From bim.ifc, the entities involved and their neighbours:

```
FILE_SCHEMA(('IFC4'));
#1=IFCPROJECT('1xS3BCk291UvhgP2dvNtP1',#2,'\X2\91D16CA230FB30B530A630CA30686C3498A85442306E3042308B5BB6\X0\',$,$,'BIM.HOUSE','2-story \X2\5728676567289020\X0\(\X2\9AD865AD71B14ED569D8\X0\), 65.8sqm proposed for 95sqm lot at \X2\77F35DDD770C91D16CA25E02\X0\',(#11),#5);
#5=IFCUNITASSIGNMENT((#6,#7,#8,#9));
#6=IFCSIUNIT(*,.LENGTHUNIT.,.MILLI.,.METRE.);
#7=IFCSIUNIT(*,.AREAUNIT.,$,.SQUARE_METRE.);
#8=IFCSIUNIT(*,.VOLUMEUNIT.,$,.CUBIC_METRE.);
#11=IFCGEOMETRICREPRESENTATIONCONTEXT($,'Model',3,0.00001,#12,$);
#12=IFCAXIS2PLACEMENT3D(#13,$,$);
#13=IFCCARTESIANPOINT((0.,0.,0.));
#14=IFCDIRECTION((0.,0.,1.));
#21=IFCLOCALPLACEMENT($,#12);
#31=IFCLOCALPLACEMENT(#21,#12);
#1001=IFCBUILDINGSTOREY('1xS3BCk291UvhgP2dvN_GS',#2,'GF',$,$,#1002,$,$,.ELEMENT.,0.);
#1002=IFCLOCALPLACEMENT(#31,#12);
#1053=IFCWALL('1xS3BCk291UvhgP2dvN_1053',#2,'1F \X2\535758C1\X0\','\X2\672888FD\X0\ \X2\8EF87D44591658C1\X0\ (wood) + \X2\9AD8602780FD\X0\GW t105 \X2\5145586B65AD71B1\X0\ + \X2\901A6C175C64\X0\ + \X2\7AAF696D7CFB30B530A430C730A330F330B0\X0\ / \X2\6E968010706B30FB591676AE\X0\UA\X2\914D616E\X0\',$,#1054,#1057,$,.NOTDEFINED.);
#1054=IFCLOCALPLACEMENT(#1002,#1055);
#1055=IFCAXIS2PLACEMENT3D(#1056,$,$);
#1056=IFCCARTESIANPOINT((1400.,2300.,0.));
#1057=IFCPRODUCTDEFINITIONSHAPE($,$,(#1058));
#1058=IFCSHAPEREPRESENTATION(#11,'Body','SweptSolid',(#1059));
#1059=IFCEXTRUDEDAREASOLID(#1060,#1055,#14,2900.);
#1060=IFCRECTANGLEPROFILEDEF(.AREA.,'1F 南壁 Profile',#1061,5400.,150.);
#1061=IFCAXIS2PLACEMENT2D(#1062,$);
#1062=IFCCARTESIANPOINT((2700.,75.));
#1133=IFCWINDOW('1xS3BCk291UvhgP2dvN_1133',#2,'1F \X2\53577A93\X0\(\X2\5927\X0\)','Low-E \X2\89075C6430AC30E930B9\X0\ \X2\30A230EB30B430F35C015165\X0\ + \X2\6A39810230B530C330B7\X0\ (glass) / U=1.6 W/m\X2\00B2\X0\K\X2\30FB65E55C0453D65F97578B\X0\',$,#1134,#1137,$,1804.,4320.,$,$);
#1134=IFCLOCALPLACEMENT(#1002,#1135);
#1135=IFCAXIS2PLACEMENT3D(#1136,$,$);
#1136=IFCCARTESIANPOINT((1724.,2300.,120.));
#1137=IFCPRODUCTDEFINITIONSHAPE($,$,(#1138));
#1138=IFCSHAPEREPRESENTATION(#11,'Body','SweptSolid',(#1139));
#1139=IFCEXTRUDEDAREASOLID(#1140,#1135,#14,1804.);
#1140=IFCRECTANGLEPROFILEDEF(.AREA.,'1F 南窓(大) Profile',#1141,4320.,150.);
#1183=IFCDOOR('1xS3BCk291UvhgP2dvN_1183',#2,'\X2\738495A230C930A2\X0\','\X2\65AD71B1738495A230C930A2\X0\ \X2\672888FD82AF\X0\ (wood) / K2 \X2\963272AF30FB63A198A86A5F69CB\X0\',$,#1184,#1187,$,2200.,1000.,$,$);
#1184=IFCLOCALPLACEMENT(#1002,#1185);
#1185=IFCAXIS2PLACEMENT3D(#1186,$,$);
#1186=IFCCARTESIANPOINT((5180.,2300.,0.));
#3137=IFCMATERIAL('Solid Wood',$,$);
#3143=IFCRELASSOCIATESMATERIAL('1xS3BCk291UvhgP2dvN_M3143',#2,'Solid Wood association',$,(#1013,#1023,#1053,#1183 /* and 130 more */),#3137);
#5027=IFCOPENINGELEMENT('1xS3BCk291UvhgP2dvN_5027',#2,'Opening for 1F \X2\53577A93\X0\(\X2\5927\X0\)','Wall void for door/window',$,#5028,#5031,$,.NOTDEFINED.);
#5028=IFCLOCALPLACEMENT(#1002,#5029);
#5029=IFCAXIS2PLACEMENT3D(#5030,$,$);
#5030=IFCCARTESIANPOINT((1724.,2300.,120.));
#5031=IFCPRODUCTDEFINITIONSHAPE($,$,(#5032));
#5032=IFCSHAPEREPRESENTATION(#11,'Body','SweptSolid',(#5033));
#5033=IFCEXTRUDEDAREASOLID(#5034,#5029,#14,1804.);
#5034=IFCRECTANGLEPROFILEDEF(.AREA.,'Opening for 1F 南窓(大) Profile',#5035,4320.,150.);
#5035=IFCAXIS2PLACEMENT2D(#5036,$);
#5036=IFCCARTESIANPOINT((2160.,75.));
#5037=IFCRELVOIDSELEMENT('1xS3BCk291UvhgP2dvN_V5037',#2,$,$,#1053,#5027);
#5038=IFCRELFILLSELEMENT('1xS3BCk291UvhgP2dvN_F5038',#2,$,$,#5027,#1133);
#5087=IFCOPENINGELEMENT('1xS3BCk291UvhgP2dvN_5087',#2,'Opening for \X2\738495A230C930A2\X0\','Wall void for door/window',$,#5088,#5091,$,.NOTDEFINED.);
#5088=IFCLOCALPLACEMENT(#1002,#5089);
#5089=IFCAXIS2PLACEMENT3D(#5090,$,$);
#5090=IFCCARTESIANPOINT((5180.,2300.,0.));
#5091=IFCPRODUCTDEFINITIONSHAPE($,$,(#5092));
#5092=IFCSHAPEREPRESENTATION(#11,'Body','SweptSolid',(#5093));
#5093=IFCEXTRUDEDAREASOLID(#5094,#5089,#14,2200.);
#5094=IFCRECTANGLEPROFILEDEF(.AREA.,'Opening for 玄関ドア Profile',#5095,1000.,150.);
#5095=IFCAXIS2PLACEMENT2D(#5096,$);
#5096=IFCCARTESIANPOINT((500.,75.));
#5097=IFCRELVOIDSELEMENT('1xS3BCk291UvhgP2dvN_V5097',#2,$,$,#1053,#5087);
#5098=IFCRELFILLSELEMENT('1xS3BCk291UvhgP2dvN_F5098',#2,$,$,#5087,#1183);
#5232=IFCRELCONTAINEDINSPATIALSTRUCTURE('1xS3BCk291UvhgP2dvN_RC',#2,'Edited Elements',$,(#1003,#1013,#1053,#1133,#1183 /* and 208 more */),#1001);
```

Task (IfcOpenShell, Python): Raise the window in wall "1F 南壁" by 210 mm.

```python
import numpy as np
import ifcopenshell
import ifcopenshell.api.geometry
import ifcopenshell.util.placement
import ifcopenshell.util.unit

model = ifcopenshell.open("bim.ifc")
unit_scale = ifcopenshell.util.unit.calculate_unit_scale(model)

window = model.by_id(1133)
opening = window.FillsVoids[0].RelatingOpeningElement
dz = 0.21 / unit_scale

shift = np.array([0.0, 0.0, dz])
# The window is not placed relative to its opening, so move both.
for product in (opening, window):
    matrix = ifcopenshell.util.placement.get_local_placement(product.ObjectPlacement)
    matrix[:3, 3] += shift
    ifcopenshell.api.geometry.edit_object_placement(model, product=product, matrix=matrix, is_si=False)

print(f"moved by {dz * unit_scale:+.3f} m")

model.write("bim_rev.ifc")
```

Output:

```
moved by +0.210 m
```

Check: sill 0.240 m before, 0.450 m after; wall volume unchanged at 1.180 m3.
